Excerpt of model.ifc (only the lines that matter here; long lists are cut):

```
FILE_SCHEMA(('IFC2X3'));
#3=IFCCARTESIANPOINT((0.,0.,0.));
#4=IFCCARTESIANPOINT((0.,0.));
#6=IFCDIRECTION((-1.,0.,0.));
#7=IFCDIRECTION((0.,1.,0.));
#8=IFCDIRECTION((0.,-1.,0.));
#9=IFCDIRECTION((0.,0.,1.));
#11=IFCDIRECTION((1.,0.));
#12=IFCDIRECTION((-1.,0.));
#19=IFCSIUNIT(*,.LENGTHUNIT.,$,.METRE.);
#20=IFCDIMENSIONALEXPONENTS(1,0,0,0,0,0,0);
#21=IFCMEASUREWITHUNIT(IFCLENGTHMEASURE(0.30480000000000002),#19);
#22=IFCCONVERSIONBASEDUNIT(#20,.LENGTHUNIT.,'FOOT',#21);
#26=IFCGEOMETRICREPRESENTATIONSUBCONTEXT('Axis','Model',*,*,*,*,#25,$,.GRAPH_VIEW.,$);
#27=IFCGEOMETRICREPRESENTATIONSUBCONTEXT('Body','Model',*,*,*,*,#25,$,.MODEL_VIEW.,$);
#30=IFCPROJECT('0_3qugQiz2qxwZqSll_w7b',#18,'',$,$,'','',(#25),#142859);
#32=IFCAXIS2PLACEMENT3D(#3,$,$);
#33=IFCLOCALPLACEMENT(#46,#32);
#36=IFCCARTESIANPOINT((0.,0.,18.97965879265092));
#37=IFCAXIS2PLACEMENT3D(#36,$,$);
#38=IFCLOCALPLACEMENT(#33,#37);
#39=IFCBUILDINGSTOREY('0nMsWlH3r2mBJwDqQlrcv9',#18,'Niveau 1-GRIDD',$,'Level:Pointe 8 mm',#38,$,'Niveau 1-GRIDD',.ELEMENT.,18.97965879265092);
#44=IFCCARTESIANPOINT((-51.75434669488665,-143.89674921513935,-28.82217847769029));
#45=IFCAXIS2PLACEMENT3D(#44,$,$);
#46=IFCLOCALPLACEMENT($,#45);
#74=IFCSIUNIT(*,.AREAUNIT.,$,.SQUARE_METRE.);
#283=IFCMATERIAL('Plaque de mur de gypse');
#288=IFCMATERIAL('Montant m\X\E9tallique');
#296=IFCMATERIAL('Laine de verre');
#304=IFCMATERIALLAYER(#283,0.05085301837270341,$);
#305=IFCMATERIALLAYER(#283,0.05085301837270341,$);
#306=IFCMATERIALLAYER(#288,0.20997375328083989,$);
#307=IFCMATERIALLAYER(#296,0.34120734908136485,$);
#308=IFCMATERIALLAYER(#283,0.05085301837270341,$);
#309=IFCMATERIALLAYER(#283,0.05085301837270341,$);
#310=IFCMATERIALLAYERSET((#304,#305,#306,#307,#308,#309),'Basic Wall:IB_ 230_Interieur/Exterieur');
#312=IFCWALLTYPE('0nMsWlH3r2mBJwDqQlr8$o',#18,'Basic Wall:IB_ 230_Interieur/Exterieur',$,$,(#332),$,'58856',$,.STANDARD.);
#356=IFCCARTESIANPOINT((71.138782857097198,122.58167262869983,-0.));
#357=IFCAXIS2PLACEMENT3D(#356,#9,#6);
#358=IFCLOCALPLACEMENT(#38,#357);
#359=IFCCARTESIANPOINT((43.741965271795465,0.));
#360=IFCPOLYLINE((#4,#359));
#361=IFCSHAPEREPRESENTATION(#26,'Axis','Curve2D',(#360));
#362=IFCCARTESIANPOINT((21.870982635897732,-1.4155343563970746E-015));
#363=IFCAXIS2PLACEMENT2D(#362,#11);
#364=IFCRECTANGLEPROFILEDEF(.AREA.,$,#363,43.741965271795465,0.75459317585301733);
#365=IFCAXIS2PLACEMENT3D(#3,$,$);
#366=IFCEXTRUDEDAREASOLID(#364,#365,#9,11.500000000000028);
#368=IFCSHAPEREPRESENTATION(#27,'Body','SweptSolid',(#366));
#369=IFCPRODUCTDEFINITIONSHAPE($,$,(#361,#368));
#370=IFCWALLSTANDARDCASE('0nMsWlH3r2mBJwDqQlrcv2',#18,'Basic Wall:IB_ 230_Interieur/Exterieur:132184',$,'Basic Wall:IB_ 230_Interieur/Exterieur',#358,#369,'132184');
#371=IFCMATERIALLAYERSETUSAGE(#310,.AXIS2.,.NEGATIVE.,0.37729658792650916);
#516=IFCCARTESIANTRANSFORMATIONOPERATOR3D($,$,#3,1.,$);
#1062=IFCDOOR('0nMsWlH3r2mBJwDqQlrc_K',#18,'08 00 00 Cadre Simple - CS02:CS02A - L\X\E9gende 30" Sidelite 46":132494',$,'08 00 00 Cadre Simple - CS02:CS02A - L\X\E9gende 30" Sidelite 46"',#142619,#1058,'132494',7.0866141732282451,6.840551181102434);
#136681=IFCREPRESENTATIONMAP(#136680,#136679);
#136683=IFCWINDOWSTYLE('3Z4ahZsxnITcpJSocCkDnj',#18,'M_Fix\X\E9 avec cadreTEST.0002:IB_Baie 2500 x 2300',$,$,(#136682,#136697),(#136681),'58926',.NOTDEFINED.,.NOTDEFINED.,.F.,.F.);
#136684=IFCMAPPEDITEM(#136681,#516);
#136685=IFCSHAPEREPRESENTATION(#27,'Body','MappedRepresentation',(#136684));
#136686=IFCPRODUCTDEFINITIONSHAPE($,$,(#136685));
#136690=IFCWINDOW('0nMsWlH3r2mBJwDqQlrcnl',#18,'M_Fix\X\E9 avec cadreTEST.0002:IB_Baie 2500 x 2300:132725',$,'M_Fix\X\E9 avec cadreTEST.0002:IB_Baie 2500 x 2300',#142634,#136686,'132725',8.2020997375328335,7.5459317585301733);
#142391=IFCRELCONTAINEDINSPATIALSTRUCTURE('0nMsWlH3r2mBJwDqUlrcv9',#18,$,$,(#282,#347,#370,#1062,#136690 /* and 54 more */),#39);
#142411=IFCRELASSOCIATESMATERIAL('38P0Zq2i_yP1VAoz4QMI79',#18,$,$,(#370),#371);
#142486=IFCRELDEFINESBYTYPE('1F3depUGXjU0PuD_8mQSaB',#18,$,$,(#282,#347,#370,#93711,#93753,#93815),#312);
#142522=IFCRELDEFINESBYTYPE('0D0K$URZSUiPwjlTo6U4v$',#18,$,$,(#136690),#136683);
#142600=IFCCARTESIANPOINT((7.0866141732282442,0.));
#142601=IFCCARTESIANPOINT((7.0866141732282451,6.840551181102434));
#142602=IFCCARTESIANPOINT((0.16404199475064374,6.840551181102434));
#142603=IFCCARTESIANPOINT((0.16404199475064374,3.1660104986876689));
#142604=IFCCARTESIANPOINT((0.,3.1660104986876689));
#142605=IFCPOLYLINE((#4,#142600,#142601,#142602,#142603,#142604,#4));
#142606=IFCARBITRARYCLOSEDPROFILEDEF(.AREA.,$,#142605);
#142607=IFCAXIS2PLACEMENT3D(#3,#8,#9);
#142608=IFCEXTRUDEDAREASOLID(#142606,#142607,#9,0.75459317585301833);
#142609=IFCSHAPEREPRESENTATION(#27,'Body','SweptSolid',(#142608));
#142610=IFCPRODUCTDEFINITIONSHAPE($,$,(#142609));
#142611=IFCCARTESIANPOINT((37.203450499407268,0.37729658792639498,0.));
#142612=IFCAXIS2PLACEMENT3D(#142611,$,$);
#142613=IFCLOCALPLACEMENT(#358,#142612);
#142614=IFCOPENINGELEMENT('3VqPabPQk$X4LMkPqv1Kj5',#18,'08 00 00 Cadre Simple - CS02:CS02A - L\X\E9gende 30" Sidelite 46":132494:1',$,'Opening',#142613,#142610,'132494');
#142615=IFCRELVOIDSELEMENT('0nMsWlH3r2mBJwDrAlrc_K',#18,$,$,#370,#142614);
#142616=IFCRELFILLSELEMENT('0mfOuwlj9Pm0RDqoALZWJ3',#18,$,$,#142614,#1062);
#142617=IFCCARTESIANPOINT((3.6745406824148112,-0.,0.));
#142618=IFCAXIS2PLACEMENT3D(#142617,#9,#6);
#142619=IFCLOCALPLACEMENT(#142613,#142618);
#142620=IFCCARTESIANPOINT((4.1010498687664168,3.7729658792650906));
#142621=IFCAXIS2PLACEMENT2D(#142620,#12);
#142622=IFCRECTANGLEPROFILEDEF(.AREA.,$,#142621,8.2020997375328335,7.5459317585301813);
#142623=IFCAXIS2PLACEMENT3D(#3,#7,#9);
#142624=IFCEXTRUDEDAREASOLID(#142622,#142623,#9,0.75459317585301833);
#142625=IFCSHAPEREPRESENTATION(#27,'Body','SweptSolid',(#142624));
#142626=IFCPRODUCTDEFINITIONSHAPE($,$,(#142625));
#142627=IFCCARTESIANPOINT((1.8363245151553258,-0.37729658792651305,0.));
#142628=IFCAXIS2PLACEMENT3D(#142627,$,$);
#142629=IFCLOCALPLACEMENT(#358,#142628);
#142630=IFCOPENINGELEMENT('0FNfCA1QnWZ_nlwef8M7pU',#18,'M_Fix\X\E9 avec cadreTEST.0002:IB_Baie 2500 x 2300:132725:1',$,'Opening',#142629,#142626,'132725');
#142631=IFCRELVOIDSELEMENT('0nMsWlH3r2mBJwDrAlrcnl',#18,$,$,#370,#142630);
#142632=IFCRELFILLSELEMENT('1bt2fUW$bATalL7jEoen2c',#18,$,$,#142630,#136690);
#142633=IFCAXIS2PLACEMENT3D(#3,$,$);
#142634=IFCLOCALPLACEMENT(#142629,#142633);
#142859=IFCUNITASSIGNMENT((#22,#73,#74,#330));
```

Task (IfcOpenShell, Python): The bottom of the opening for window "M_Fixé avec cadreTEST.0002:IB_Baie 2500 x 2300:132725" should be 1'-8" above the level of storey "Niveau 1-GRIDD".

```python
import numpy as np
import ifcopenshell
import ifcopenshell.api.geometry
import ifcopenshell.geom
import ifcopenshell.util.element
import ifcopenshell.util.placement
import ifcopenshell.util.shape
import ifcopenshell.util.unit

model = ifcopenshell.open("model.ifc")
unit_scale = ifcopenshell.util.unit.calculate_unit_scale(model)

window = model.by_guid("0nMsWlH3r2mBJwDqQlrcnl")
opening = window.FillsVoids[0].RelatingOpeningElement
storey = ifcopenshell.util.element.get_container(window, ifc_class="IfcBuildingStorey")
level = ifcopenshell.util.placement.get_local_placement(storey.ObjectPlacement)[2, 3]

# The opening's origin need not be at the sill, so measure its lowest point.
shape = ifcopenshell.geom.create_shape(ifcopenshell.geom.settings(), opening)
bottom = ifcopenshell.util.shape.get_shape_bottom_elevation(shape, shape.geometry) / unit_scale
dz = level + 20 * 0.0254 / unit_scale - bottom

shift = np.array([0.0, 0.0, dz])
# The window is placed relative to its opening, so it follows when the opening moves.
matrix = ifcopenshell.util.placement.get_local_placement(opening.ObjectPlacement)
matrix[:3, 3] += shift
ifcopenshell.api.geometry.edit_object_placement(
    model, product=opening, matrix=matrix, is_si=False, should_transform_children=True
)

print(f"moved by {dz * unit_scale:+.3f} m")

model.write("model_edited.ifc")
```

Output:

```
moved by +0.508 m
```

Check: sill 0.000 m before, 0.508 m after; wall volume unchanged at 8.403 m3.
